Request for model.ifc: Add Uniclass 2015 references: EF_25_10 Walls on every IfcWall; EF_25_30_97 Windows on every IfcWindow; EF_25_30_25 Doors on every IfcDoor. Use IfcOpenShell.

First a look at what the model holds.

```python
import ifcopenshell

model = ifcopenshell.open("model.ifc")
print(model.schema)
print("classifications:", [c.Name for c in model.by_type("IfcClassification")])
for ifc_class in ("IfcDoor", "IfcRoof", "IfcStair", "IfcWall", "IfcWindow"):
    print(ifc_class, len(model.by_type(ifc_class)))
```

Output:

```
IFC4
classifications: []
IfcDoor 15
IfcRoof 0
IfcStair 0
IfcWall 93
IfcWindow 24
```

```python
import ifcopenshell
import ifcopenshell.api.classification

model = ifcopenshell.open("model.ifc")

system = ifcopenshell.api.classification.add_classification(model, classification="Uniclass 2015")

codes = {
    "IfcWall": ("EF_25_10", "Walls"),
    "IfcWindow": ("EF_25_30_97", "Windows"),
    "IfcDoor": ("EF_25_30_25", "Doors"),
}
for ifc_class, (code, name) in codes.items():
    products = model.by_type(ifc_class)
    ifcopenshell.api.classification.add_reference(
        model, products=products, classification=system, identification=code, name=name
    )
    print(code, len(products))

model.write("model_rev.ifc")
```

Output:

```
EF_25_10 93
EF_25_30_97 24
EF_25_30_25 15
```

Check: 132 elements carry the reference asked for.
